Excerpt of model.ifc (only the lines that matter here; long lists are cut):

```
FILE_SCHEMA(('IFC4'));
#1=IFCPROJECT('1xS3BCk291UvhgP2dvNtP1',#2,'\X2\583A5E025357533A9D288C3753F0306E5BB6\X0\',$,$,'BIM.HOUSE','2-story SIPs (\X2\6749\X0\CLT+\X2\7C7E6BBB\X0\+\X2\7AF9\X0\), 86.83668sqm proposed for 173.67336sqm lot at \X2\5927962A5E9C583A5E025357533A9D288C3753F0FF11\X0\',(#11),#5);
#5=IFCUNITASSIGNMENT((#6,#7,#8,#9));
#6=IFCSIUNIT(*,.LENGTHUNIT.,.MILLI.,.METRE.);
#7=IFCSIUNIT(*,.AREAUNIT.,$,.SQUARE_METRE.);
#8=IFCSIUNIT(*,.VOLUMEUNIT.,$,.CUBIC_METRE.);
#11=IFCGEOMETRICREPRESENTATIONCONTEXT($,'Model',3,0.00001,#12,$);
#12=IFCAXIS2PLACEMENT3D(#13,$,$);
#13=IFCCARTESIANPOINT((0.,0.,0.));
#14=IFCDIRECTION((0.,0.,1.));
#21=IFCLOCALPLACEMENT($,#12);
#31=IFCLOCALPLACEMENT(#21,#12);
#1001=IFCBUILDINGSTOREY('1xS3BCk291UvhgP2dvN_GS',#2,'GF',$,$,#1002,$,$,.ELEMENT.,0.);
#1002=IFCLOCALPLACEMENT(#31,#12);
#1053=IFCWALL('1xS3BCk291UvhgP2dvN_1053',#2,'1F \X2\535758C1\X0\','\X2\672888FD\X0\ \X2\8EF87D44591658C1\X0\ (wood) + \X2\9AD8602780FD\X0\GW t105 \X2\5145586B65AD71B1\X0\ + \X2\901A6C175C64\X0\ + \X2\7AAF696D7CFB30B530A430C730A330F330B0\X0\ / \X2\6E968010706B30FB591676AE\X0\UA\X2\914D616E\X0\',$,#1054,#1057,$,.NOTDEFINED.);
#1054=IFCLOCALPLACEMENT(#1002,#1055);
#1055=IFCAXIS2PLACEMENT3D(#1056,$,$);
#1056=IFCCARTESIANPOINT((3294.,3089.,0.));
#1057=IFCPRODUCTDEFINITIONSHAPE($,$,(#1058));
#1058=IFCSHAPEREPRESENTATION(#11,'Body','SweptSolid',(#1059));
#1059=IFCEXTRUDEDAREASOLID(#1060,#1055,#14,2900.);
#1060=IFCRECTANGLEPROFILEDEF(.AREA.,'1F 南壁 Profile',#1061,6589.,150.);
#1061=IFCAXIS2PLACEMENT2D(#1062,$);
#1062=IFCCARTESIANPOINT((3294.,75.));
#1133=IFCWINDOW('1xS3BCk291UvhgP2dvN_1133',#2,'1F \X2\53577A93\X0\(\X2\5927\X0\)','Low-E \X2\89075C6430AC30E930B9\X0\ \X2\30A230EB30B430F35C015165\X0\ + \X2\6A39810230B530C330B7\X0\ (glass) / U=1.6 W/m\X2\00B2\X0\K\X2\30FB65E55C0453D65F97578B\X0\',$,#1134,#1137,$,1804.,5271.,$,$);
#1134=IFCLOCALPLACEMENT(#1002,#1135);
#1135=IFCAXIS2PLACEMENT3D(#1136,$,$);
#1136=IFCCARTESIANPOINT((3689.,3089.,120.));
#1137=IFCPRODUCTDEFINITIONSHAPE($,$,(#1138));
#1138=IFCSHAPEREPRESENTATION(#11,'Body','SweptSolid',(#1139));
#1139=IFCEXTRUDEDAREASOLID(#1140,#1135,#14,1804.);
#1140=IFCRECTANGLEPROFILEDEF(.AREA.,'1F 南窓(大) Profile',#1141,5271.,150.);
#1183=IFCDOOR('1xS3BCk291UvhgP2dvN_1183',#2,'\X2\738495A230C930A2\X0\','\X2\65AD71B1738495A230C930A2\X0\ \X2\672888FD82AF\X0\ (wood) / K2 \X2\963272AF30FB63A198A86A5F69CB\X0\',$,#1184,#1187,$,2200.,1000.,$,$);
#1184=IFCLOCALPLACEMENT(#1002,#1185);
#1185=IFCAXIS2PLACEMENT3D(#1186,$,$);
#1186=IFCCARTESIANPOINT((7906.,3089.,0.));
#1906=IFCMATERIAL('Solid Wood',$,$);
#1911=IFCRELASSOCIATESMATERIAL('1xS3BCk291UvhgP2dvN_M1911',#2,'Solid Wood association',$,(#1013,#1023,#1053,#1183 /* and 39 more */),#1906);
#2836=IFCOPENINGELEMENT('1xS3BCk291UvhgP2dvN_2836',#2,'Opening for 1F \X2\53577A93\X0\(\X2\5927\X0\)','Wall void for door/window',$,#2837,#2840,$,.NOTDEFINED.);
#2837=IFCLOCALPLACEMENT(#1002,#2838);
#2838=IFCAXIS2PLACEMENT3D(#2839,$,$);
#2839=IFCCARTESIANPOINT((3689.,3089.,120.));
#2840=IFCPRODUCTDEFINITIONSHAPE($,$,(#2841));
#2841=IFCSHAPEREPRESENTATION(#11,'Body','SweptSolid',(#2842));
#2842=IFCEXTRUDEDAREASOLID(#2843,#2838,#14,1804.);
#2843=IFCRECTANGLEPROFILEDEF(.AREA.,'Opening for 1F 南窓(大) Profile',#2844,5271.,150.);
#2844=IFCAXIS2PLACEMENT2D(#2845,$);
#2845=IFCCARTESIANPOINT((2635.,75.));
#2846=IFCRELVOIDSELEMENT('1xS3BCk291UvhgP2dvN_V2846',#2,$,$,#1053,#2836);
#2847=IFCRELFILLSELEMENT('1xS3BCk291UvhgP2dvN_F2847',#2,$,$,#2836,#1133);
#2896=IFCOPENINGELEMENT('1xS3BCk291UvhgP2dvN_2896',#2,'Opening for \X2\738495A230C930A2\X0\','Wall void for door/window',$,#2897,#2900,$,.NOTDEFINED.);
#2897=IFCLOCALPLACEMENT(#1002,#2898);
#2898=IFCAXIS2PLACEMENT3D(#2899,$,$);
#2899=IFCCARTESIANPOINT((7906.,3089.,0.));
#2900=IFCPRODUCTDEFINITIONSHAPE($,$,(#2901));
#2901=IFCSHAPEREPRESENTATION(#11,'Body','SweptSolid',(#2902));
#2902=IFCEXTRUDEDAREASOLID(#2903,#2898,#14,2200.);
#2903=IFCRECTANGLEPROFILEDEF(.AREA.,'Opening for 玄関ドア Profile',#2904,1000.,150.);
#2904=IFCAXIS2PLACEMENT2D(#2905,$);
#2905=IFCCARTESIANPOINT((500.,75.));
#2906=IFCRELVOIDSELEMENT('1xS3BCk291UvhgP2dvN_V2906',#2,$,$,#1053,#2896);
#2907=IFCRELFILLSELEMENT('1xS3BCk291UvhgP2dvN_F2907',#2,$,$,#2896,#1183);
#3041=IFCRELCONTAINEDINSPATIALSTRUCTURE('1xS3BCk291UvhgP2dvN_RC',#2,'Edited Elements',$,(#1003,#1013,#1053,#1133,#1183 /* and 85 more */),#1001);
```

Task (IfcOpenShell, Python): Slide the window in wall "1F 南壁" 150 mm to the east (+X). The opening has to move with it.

```python
import ifcopenshell
import ifcopenshell.api.geometry
import ifcopenshell.util.placement

model = ifcopenshell.open("model.ifc")

window = model.by_guid("1xS3BCk291UvhgP2dvN_1133")
opening = window.FillsVoids[0].RelatingOpeningElement
wall = opening.VoidsElements[0].RelatingBuildingElement

wall_matrix = ifcopenshell.util.placement.get_local_placement(wall.ObjectPlacement)
shift = wall_matrix[:3, 0] * 150.0
before = ifcopenshell.util.placement.get_local_placement(window.ObjectPlacement)[:3, 3].copy()

# The window is not placed relative to its opening, so move both.
for product in (opening, window):
    matrix = ifcopenshell.util.placement.get_local_placement(product.ObjectPlacement)
    matrix[:3, 3] += shift
    ifcopenshell.api.geometry.edit_object_placement(model, product=product, matrix=matrix, is_si=False)

after = ifcopenshell.util.placement.get_local_placement(window.ObjectPlacement)[:3, 3]
print("window moved by", (after - before).round(3) + 0.0)

model.write("model_rev.ifc")
```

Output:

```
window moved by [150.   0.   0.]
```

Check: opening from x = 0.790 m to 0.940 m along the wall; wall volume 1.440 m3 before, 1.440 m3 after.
